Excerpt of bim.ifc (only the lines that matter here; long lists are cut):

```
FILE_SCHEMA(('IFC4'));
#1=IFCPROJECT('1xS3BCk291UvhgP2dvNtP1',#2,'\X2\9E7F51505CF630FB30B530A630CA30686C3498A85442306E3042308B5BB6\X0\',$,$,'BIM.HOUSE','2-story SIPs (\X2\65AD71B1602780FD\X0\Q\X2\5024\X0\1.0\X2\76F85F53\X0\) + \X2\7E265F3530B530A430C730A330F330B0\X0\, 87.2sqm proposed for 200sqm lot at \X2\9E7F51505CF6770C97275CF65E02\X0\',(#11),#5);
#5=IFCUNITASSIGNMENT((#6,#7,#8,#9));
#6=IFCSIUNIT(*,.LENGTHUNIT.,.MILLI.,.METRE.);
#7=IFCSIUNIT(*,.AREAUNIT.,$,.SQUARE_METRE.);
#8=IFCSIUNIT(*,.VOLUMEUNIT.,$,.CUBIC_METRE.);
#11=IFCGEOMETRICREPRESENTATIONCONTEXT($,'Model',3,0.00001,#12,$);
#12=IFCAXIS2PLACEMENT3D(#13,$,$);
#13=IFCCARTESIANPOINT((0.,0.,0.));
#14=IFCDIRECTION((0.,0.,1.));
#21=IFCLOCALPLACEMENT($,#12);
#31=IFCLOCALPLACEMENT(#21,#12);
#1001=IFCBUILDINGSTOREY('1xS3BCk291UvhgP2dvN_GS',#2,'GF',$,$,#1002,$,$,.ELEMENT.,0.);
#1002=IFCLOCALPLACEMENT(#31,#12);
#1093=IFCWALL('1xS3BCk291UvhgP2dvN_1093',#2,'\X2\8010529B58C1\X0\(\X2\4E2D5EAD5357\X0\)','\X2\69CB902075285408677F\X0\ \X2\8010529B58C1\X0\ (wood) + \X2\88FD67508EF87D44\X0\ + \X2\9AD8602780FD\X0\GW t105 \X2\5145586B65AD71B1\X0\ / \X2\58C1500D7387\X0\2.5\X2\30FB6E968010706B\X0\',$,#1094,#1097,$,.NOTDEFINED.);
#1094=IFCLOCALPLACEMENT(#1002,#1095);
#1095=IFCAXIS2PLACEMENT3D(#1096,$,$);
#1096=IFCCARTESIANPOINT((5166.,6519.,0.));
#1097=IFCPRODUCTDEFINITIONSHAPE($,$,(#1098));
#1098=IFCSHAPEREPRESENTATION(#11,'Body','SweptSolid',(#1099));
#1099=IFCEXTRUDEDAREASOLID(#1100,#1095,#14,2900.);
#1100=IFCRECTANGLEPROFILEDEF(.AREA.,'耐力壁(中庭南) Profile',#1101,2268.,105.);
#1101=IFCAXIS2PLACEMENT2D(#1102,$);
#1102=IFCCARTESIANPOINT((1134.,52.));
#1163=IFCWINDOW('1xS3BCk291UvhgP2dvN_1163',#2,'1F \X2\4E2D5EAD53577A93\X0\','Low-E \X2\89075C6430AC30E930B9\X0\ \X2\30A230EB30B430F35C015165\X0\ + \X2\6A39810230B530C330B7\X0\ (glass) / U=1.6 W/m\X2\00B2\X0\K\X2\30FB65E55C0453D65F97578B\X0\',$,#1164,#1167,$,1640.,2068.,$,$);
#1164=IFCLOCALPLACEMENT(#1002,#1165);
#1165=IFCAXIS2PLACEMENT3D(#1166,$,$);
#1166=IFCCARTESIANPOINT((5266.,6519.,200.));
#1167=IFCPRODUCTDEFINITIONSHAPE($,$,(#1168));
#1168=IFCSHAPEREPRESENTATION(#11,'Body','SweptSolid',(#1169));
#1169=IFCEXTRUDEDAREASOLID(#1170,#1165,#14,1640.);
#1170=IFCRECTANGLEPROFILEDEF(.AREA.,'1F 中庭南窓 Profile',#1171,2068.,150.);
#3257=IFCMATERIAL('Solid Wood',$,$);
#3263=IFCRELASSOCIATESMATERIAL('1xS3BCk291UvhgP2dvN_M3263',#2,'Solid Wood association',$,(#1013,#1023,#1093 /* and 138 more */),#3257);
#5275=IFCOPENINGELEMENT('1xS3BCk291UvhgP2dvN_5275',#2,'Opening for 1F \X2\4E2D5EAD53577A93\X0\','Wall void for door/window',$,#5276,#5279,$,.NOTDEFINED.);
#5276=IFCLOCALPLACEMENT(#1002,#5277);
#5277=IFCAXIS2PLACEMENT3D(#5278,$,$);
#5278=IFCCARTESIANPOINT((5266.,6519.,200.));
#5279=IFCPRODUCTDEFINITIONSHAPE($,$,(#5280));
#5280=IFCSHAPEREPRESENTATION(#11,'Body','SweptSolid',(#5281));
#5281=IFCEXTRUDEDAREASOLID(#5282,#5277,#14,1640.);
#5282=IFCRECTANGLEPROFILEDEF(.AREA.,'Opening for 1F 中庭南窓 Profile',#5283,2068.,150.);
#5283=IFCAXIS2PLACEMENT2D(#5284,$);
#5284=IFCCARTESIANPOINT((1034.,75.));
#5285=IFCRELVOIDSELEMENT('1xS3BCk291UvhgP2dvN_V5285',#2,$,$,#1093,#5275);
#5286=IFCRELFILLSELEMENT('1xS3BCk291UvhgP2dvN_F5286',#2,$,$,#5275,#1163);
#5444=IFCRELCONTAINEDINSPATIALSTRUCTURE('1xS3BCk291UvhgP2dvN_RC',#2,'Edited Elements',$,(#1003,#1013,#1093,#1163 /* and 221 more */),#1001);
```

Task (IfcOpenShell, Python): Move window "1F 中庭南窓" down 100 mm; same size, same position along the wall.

```python
import numpy as np
import ifcopenshell
import ifcopenshell.api.geometry
import ifcopenshell.util.placement
import ifcopenshell.util.unit

model = ifcopenshell.open("bim.ifc")
unit_scale = ifcopenshell.util.unit.calculate_unit_scale(model)

window = model.by_guid("1xS3BCk291UvhgP2dvN_1163")
opening = window.FillsVoids[0].RelatingOpeningElement
dz = -0.1 / unit_scale

shift = np.array([0.0, 0.0, dz])
# The window is not placed relative to its opening, so move both.
for product in (opening, window):
    matrix = ifcopenshell.util.placement.get_local_placement(product.ObjectPlacement)
    matrix[:3, 3] += shift
    ifcopenshell.api.geometry.edit_object_placement(model, product=product, matrix=matrix, is_si=False)

print(f"moved by {dz * unit_scale:+.3f} m")

model.write("bim-out.ifc")
```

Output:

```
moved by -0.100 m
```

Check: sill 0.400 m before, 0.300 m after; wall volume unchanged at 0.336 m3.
